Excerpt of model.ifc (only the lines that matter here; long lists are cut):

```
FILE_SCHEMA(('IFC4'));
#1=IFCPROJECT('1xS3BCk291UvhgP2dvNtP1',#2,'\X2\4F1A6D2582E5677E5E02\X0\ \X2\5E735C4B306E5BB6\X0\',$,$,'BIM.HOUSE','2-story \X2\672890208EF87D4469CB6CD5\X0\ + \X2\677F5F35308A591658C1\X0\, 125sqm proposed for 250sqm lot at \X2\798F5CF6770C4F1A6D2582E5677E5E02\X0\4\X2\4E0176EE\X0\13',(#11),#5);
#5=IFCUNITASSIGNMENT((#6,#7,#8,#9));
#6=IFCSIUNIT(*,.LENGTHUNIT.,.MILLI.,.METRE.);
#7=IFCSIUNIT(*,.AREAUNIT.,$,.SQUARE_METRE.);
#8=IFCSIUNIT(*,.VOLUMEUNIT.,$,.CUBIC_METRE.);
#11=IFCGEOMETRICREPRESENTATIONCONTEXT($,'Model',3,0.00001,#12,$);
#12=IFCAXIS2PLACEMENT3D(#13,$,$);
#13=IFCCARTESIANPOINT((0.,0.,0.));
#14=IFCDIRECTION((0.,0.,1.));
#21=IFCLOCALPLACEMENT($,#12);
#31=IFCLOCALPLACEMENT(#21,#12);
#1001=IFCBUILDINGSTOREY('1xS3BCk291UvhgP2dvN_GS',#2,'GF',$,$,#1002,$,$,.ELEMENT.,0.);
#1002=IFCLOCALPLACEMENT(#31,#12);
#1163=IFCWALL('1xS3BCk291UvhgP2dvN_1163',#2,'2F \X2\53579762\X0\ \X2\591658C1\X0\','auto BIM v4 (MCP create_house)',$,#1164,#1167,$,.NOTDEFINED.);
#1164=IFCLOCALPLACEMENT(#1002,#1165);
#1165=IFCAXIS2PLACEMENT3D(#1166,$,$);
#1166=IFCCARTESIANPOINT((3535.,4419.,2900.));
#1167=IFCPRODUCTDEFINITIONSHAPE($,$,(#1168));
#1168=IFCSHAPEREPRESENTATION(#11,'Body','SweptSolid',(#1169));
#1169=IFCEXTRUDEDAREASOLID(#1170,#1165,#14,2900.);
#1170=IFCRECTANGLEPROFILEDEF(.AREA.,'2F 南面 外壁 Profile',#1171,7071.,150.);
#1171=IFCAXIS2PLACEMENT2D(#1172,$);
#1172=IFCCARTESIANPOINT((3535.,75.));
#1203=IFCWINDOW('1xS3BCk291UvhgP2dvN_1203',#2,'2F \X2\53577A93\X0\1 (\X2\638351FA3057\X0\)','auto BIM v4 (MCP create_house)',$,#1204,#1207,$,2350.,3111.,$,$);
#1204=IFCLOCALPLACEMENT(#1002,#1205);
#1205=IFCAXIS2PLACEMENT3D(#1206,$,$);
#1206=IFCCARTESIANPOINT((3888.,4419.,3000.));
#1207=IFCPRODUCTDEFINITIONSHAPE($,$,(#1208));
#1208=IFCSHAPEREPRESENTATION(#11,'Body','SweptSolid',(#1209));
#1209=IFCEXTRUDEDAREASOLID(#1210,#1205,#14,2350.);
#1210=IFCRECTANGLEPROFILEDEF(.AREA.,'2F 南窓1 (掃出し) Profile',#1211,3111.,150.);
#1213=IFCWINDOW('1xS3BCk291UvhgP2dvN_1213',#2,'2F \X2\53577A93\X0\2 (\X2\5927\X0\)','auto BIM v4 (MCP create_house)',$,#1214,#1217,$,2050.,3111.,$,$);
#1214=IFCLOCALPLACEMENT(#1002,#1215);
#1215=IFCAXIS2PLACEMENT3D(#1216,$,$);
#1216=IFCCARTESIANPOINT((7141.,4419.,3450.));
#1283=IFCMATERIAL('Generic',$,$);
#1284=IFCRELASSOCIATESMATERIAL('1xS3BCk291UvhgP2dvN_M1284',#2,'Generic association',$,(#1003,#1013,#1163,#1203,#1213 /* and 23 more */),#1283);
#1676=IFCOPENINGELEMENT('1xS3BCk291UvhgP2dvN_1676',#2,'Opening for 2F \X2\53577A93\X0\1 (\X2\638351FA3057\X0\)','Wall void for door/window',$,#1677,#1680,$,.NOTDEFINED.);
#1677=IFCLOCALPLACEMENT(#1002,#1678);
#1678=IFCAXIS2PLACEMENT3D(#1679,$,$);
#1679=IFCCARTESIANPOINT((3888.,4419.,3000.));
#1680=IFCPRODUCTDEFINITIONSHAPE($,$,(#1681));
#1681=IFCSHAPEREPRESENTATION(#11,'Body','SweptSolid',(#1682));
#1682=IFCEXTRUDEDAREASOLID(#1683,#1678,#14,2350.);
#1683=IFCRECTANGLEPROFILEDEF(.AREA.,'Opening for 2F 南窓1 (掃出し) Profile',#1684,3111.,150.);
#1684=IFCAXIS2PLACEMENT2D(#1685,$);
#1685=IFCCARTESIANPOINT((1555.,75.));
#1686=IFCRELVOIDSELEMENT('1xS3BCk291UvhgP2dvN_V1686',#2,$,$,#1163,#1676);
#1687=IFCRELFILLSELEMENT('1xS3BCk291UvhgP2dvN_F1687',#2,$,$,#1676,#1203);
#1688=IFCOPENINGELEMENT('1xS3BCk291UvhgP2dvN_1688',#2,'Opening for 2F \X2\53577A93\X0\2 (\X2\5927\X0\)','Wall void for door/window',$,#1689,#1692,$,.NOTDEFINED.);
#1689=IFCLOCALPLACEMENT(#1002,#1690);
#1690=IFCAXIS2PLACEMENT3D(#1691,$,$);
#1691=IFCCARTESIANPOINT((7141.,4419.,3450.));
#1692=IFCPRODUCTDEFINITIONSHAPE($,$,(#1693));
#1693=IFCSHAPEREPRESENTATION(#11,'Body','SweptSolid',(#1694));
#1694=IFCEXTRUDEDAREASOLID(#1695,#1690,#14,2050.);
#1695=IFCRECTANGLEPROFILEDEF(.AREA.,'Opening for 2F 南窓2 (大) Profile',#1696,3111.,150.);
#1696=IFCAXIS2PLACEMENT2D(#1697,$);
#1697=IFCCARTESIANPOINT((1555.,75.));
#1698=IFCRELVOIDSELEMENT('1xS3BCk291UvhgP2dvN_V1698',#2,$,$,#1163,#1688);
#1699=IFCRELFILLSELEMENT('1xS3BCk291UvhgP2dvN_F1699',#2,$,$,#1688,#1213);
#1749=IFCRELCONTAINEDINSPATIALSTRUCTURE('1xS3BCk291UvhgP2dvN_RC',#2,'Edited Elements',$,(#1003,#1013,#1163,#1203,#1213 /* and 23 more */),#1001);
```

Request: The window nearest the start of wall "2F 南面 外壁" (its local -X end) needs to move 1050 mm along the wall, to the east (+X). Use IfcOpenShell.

```python
import ifcopenshell
import ifcopenshell.api.geometry
import ifcopenshell.util.placement
import ifcopenshell.util.unit

model = ifcopenshell.open("model.ifc")
unit_scale = ifcopenshell.util.unit.calculate_unit_scale(model)

window = model.by_guid("1xS3BCk291UvhgP2dvN_1203")
opening = window.FillsVoids[0].RelatingOpeningElement
wall = opening.VoidsElements[0].RelatingBuildingElement

wall_matrix = ifcopenshell.util.placement.get_local_placement(wall.ObjectPlacement)
shift = wall_matrix[:3, 0] * 1.05 / unit_scale
before = ifcopenshell.util.placement.get_local_placement(window.ObjectPlacement)[:3, 3].copy()

# The window is not placed relative to its opening, so move both.
for product in (opening, window):
    matrix = ifcopenshell.util.placement.get_local_placement(product.ObjectPlacement)
    matrix[:3, 3] += shift
    ifcopenshell.api.geometry.edit_object_placement(model, product=product, matrix=matrix, is_si=False)

after = ifcopenshell.util.placement.get_local_placement(window.ObjectPlacement)[:3, 3]
print("window moved by", (after - before).round(3) + 0.0)

model.write("model-out.ifc")
```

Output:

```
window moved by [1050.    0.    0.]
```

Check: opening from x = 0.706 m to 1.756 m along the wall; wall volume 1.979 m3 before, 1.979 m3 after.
